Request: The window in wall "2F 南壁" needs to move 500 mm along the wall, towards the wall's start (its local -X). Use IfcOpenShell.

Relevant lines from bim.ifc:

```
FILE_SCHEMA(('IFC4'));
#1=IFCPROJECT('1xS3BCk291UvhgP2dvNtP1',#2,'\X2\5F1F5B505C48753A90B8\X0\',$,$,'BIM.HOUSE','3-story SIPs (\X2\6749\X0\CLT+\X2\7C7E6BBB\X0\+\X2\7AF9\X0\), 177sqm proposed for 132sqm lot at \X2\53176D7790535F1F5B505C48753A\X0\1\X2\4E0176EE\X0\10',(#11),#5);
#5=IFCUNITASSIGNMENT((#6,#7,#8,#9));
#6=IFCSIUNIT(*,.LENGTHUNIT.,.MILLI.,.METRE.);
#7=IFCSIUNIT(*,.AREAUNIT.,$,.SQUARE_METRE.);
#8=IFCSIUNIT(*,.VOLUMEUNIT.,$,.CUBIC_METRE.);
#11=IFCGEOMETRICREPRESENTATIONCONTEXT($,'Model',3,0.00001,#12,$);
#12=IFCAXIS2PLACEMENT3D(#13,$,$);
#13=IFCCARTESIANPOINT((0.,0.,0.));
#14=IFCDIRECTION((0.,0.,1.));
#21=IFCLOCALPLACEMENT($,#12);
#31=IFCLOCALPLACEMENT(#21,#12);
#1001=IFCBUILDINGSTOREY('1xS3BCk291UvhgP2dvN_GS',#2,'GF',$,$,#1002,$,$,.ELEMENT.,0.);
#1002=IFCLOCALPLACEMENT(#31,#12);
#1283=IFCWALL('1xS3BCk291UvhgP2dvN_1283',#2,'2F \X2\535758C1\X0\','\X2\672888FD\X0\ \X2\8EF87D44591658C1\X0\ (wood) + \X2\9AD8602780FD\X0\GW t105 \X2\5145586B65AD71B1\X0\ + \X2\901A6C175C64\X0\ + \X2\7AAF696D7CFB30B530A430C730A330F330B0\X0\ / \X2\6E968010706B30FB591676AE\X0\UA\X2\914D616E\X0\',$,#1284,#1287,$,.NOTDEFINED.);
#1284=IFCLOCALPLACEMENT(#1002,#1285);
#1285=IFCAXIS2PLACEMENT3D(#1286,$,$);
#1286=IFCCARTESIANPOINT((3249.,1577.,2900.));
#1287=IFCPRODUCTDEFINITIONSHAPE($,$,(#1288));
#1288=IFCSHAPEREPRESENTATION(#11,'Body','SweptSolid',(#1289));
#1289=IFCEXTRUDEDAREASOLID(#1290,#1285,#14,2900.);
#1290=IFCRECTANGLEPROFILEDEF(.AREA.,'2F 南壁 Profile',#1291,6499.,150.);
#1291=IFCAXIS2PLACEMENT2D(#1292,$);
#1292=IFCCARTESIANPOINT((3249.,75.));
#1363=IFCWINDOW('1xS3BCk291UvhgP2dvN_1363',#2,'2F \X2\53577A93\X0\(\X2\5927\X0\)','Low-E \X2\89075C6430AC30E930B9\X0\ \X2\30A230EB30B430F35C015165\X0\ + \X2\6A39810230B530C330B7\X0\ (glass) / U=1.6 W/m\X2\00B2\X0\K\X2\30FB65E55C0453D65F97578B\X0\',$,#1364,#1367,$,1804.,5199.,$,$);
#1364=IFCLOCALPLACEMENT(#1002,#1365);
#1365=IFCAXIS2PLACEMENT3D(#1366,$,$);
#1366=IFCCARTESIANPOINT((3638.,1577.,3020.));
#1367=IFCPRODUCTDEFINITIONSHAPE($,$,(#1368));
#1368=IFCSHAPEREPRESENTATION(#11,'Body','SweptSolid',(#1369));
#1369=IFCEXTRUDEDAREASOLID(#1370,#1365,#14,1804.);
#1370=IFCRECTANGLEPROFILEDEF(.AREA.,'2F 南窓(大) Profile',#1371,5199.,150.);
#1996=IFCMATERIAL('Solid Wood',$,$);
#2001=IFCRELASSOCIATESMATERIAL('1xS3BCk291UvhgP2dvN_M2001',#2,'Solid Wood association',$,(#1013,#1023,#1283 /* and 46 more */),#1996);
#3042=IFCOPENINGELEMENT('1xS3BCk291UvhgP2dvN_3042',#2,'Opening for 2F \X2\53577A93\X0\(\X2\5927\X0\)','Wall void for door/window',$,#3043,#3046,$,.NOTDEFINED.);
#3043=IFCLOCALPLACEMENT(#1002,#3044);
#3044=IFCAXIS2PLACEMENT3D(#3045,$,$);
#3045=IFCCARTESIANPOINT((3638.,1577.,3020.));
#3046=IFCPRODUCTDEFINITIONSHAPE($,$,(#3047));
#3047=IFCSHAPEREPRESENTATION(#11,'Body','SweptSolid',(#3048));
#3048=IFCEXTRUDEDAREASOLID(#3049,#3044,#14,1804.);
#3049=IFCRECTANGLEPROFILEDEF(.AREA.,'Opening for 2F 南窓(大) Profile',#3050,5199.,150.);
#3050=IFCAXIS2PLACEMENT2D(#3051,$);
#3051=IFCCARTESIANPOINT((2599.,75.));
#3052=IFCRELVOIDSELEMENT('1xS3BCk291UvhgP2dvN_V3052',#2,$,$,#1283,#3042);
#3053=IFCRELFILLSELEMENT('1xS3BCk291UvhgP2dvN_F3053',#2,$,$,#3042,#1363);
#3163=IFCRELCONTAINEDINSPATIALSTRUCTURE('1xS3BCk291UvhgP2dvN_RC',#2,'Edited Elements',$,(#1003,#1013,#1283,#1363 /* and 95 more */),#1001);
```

```python
import ifcopenshell
import ifcopenshell.api.geometry
import ifcopenshell.util.placement

model = ifcopenshell.open("bim.ifc")

window = model.by_guid("1xS3BCk291UvhgP2dvN_1363")
opening = window.FillsVoids[0].RelatingOpeningElement
wall = opening.VoidsElements[0].RelatingBuildingElement

wall_matrix = ifcopenshell.util.placement.get_local_placement(wall.ObjectPlacement)
shift = wall_matrix[:3, 0] * -500.0
before = ifcopenshell.util.placement.get_local_placement(window.ObjectPlacement)[:3, 3].copy()

# The window is not placed relative to its opening, so move both.
for product in (opening, window):
    matrix = ifcopenshell.util.placement.get_local_placement(product.ObjectPlacement)
    matrix[:3, 3] += shift
    ifcopenshell.api.geometry.edit_object_placement(model, product=product, matrix=matrix, is_si=False)

after = ifcopenshell.util.placement.get_local_placement(window.ObjectPlacement)[:3, 3]
print("window moved by", (after - before).round(3) + 0.0)

model.write("bim_updated.ifc")
```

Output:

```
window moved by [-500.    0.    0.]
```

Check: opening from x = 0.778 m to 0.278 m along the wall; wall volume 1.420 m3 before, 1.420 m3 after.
